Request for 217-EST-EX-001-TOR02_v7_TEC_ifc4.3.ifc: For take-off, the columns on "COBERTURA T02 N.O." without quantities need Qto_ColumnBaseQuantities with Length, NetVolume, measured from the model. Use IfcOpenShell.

First a look at what the model holds.

```python
import ifcopenshell
import ifcopenshell.util.element
import ifcopenshell.util.unit

model = ifcopenshell.open("217-EST-EX-001-TOR02_v7_TEC_ifc4.3.ifc")
print(model.schema)
for unit_type in ("LENGTHUNIT", "AREAUNIT", "VOLUMEUNIT"):
    print(unit_type, ifcopenshell.util.unit.calculate_unit_scale(model, unit_type))
storey = next(s for s in model.by_type("IfcBuildingStorey") if s.Name == "COBERTURA T02 N.O.")
columns = [e for e in ifcopenshell.util.element.get_decomposition(storey) if e.is_a("IfcColumn")]
for e in sorted(columns, key=lambda e: e.id()):
    print(e.id(), e.is_a(), e.Name, list(ifcopenshell.util.element.get_psets(e, qtos_only=True)), sep=" | ")
```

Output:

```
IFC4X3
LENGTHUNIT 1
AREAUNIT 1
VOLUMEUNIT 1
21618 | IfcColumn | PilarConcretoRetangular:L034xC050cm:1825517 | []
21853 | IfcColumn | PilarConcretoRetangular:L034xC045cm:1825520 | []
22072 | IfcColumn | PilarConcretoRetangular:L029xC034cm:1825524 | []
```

```python
import ifcopenshell
import ifcopenshell.api.pset
import ifcopenshell.geom
import ifcopenshell.util.element
import ifcopenshell.util.shape
import ifcopenshell.util.unit

model = ifcopenshell.open("217-EST-EX-001-TOR02_v7_TEC_ifc4.3.ifc")
unit_scale = ifcopenshell.util.unit.calculate_unit_scale(model)
volume_scale = ifcopenshell.util.unit.calculate_unit_scale(model, "VOLUMEUNIT")
settings = ifcopenshell.geom.settings()

storey = next(s for s in model.by_type("IfcBuildingStorey") if s.Name == "COBERTURA T02 N.O.")
columns = [e for e in ifcopenshell.util.element.get_decomposition(storey) if e.is_a("IfcColumn")]

for e in sorted(columns, key=lambda e: e.id()):
    if ifcopenshell.util.element.get_psets(e, qtos_only=True, should_inherit=False):
        continue
    # Geometry comes back in metres, in the element's own axes.
    shape = ifcopenshell.geom.create_shape(settings, e)
    values = {
        "Length": ifcopenshell.util.shape.get_z(shape.geometry) / unit_scale,
        "NetVolume": ifcopenshell.util.shape.get_volume(shape.geometry) / volume_scale,
    }
    qto = ifcopenshell.api.pset.add_qto(model, product=e, name="Qto_ColumnBaseQuantities")
    ifcopenshell.api.pset.edit_qto(model, qto=qto, properties=values)
    print(e.id(), {k: round(v, 3) for k, v in values.items()})

model.write("217-EST-EX-001-TOR02_v7_TEC_ifc4.3_v2.ifc")
```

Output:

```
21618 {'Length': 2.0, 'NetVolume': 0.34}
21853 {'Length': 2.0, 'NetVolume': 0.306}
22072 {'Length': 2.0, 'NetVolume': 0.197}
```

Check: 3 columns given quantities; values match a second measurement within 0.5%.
